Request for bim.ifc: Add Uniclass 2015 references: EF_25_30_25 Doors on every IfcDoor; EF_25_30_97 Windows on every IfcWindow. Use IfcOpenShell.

First a look at what the model holds.

```python
import ifcopenshell

model = ifcopenshell.open("bim.ifc")
print(model.schema)
print("classifications:", [c.Name for c in model.by_type("IfcClassification")])
for ifc_class in ("IfcDoor", "IfcRoof", "IfcStair", "IfcWall", "IfcWindow"):
    print(ifc_class, len(model.by_type(ifc_class)))
```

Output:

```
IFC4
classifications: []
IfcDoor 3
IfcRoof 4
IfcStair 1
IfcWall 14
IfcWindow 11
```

```python
import ifcopenshell
import ifcopenshell.api.classification

model = ifcopenshell.open("bim.ifc")

system = ifcopenshell.api.classification.add_classification(model, classification="Uniclass 2015")

codes = {
    "IfcDoor": ("EF_25_30_25", "Doors"),
    "IfcWindow": ("EF_25_30_97", "Windows"),
}
for ifc_class, (code, name) in codes.items():
    products = model.by_type(ifc_class)
    ifcopenshell.api.classification.add_reference(
        model, products=products, classification=system, identification=code, name=name
    )
    print(code, len(products))

model.write("bim_v2.ifc")
```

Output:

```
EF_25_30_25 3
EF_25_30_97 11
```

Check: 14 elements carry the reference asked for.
